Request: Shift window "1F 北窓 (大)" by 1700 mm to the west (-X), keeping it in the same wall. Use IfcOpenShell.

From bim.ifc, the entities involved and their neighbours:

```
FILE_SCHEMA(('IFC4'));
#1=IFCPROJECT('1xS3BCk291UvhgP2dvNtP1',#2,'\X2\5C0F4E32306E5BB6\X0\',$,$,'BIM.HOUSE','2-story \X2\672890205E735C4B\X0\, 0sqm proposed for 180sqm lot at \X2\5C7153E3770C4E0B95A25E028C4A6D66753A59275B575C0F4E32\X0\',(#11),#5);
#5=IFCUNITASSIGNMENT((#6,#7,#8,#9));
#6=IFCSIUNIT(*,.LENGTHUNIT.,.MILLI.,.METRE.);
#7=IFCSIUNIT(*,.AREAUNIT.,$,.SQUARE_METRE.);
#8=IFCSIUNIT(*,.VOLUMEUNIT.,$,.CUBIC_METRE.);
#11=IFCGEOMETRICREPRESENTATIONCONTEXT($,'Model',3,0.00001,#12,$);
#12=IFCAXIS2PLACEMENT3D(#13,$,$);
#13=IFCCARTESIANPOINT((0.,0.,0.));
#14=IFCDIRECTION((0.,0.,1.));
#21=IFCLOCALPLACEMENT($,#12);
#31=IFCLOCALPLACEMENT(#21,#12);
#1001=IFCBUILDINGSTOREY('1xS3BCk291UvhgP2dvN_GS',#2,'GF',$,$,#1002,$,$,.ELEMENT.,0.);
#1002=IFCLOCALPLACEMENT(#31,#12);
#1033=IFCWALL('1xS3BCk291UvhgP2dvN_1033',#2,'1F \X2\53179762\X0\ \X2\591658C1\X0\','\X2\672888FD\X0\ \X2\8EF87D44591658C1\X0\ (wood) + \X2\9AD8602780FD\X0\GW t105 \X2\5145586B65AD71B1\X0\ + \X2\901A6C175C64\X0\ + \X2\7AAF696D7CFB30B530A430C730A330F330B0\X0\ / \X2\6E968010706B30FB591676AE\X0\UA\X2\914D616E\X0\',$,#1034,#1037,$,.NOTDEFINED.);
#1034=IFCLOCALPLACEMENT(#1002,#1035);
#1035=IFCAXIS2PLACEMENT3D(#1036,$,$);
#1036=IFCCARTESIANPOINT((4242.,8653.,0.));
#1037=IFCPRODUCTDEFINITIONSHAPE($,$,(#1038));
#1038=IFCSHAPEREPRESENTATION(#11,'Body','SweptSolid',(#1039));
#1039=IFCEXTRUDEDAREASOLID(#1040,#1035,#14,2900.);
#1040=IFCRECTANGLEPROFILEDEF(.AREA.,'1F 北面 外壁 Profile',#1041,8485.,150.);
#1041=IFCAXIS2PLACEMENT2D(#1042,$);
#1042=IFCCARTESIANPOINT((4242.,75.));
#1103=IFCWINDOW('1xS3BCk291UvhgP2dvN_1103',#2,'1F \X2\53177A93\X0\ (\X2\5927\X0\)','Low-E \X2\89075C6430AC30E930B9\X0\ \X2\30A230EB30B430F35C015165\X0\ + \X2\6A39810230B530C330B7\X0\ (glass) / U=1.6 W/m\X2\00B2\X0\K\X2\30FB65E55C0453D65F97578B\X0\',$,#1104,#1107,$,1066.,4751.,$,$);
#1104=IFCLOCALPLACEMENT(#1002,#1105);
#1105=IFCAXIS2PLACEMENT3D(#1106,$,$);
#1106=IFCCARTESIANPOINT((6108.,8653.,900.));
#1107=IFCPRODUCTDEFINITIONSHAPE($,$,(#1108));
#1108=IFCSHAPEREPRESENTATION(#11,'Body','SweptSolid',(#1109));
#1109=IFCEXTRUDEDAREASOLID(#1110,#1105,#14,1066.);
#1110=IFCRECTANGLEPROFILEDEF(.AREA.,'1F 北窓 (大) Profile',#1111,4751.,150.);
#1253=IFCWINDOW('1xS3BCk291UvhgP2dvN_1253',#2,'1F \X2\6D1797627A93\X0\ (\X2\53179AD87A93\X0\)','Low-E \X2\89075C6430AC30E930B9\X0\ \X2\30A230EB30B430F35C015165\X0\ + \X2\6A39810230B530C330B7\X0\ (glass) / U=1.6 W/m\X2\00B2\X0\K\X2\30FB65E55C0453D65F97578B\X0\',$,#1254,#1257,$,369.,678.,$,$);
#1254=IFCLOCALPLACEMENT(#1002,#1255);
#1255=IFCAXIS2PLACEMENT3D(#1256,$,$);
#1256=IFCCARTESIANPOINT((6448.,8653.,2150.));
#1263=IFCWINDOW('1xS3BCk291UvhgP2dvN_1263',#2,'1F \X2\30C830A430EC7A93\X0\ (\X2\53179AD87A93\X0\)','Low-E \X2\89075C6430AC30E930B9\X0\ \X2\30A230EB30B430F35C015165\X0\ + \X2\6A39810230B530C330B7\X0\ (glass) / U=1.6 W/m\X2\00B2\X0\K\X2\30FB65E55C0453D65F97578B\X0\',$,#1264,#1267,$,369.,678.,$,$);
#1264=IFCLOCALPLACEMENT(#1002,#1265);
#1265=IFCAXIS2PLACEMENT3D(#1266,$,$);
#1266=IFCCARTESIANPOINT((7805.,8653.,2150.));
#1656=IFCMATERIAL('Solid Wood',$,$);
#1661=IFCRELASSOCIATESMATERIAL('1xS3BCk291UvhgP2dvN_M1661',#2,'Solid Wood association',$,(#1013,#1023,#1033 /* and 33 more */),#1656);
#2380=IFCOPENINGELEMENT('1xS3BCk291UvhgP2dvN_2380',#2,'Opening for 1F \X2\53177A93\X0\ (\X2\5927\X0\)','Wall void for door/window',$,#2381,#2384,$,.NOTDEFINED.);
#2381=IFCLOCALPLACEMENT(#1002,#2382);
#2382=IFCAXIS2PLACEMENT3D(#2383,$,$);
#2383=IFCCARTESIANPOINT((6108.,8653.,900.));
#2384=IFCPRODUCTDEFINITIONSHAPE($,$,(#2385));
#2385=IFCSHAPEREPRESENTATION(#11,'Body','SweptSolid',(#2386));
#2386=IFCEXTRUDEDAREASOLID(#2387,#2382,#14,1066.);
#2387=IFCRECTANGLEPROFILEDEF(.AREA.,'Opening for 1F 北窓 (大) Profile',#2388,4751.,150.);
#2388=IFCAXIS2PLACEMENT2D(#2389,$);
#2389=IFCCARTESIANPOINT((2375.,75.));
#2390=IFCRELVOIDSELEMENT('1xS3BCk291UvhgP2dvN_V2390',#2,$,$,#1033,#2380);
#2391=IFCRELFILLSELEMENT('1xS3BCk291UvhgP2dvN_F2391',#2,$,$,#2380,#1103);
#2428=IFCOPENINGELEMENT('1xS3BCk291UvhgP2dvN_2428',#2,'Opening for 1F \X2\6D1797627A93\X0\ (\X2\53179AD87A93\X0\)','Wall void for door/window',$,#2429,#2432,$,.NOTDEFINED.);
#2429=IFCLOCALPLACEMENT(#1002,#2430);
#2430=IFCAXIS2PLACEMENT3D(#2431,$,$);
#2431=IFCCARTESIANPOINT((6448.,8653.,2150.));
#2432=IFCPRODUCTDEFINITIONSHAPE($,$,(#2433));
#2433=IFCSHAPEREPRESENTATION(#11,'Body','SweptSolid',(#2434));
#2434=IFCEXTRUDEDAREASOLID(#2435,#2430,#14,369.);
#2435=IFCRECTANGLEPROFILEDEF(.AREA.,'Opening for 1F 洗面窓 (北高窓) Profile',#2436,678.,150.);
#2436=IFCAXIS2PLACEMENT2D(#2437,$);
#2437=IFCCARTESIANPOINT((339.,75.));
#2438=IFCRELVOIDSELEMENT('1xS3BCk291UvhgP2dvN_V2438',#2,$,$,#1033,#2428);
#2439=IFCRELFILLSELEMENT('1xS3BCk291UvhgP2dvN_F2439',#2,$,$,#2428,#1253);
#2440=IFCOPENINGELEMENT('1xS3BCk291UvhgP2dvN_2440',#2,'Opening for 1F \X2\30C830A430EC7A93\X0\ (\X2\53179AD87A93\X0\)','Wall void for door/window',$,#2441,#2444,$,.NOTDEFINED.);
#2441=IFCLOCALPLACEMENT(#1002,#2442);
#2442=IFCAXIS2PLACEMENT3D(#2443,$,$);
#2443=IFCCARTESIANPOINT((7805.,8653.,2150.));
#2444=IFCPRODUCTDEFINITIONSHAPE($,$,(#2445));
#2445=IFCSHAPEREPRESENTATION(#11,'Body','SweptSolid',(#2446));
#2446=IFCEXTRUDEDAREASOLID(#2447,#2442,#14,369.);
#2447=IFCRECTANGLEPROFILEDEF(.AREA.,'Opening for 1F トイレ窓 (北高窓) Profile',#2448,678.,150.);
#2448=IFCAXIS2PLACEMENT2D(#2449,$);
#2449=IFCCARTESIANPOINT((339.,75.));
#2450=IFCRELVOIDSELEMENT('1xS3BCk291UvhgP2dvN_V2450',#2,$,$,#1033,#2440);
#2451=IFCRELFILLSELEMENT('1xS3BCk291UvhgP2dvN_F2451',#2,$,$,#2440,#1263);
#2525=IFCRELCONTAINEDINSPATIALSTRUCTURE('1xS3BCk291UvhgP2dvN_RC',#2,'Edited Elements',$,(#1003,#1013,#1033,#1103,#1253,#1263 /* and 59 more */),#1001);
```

```python
import ifcopenshell
import ifcopenshell.api.geometry
import ifcopenshell.util.placement
import ifcopenshell.util.unit

model = ifcopenshell.open("bim.ifc")
unit_scale = ifcopenshell.util.unit.calculate_unit_scale(model)

window = model.by_id(1103)
opening = window.FillsVoids[0].RelatingOpeningElement
wall = opening.VoidsElements[0].RelatingBuildingElement

wall_matrix = ifcopenshell.util.placement.get_local_placement(wall.ObjectPlacement)
shift = wall_matrix[:3, 0] * -1.7 / unit_scale
before = ifcopenshell.util.placement.get_local_placement(window.ObjectPlacement)[:3, 3].copy()

# The window is not placed relative to its opening, so move both.
for product in (opening, window):
    matrix = ifcopenshell.util.placement.get_local_placement(product.ObjectPlacement)
    matrix[:3, 3] += shift
    ifcopenshell.api.geometry.edit_object_placement(model, product=product, matrix=matrix, is_si=False)

after = ifcopenshell.util.placement.get_local_placement(window.ObjectPlacement)[:3, 3]
print("window moved by", (after - before).round(3) + 0.0)

model.write("bim-out.ifc")
```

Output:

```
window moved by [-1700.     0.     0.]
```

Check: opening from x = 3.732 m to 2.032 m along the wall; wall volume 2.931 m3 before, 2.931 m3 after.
